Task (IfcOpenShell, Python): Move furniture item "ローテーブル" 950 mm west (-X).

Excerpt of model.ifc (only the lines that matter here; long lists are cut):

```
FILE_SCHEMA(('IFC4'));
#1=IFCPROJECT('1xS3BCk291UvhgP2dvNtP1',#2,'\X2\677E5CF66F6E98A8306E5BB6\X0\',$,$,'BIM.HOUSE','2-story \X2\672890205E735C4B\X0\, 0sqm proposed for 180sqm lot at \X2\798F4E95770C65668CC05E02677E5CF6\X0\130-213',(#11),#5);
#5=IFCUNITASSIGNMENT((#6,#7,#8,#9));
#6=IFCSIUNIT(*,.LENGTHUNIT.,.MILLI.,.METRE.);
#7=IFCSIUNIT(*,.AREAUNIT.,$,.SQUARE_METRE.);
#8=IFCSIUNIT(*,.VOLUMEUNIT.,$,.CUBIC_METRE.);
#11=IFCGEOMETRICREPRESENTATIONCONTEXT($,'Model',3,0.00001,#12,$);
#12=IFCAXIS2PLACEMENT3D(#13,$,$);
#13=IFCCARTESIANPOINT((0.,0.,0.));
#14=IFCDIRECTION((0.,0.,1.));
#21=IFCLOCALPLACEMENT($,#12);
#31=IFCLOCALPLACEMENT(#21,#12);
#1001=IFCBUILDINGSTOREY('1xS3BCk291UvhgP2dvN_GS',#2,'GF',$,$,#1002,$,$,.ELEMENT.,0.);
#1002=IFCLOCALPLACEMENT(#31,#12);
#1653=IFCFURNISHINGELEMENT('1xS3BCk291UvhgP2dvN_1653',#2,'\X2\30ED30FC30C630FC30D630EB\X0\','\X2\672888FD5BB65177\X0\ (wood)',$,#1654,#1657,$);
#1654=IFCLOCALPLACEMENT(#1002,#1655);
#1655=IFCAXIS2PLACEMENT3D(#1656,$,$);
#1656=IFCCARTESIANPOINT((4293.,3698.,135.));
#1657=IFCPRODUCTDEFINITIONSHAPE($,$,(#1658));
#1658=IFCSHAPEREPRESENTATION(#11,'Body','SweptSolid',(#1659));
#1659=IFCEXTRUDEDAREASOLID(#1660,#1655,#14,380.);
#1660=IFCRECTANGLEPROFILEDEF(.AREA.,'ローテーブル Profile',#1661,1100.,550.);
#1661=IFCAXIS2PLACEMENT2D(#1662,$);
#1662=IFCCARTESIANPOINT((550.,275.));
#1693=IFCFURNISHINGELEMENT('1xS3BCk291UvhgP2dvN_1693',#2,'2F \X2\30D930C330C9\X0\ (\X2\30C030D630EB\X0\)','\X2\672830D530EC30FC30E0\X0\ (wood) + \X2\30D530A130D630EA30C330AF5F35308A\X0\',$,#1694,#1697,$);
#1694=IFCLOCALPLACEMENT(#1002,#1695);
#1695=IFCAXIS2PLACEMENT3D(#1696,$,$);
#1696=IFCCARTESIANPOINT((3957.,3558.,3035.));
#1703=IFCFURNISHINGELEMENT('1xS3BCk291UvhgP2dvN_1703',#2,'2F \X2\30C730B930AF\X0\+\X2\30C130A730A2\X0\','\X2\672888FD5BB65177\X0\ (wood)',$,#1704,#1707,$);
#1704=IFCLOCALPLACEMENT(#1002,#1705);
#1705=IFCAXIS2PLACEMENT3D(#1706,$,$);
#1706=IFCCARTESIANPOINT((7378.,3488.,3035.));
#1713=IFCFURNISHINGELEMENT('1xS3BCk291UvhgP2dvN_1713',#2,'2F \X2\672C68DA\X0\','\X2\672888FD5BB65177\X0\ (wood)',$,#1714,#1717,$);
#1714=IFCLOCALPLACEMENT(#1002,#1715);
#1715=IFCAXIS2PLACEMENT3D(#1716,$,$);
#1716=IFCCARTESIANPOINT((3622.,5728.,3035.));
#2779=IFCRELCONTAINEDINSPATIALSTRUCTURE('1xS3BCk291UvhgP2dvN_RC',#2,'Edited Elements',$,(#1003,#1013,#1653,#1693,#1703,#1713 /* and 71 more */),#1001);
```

```python
import ifcopenshell
import ifcopenshell.api.geometry
import ifcopenshell.util.placement
import ifcopenshell.util.unit

model = ifcopenshell.open("model.ifc")
unit_scale = ifcopenshell.util.unit.calculate_unit_scale(model)

item = model.by_guid("1xS3BCk291UvhgP2dvN_1653")
matrix = ifcopenshell.util.placement.get_local_placement(item.ObjectPlacement)
matrix[0, 3] -= 0.95 / unit_scale
ifcopenshell.api.geometry.edit_object_placement(model, product=item, matrix=matrix, is_si=False)

print(ifcopenshell.util.placement.get_local_placement(item.ObjectPlacement).round(3) + 0.0)

model.write("model_updated.ifc")
```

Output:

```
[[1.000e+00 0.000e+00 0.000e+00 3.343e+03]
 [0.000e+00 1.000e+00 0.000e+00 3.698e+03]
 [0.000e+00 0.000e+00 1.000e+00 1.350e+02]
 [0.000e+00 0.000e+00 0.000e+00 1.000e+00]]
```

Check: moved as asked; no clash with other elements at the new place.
